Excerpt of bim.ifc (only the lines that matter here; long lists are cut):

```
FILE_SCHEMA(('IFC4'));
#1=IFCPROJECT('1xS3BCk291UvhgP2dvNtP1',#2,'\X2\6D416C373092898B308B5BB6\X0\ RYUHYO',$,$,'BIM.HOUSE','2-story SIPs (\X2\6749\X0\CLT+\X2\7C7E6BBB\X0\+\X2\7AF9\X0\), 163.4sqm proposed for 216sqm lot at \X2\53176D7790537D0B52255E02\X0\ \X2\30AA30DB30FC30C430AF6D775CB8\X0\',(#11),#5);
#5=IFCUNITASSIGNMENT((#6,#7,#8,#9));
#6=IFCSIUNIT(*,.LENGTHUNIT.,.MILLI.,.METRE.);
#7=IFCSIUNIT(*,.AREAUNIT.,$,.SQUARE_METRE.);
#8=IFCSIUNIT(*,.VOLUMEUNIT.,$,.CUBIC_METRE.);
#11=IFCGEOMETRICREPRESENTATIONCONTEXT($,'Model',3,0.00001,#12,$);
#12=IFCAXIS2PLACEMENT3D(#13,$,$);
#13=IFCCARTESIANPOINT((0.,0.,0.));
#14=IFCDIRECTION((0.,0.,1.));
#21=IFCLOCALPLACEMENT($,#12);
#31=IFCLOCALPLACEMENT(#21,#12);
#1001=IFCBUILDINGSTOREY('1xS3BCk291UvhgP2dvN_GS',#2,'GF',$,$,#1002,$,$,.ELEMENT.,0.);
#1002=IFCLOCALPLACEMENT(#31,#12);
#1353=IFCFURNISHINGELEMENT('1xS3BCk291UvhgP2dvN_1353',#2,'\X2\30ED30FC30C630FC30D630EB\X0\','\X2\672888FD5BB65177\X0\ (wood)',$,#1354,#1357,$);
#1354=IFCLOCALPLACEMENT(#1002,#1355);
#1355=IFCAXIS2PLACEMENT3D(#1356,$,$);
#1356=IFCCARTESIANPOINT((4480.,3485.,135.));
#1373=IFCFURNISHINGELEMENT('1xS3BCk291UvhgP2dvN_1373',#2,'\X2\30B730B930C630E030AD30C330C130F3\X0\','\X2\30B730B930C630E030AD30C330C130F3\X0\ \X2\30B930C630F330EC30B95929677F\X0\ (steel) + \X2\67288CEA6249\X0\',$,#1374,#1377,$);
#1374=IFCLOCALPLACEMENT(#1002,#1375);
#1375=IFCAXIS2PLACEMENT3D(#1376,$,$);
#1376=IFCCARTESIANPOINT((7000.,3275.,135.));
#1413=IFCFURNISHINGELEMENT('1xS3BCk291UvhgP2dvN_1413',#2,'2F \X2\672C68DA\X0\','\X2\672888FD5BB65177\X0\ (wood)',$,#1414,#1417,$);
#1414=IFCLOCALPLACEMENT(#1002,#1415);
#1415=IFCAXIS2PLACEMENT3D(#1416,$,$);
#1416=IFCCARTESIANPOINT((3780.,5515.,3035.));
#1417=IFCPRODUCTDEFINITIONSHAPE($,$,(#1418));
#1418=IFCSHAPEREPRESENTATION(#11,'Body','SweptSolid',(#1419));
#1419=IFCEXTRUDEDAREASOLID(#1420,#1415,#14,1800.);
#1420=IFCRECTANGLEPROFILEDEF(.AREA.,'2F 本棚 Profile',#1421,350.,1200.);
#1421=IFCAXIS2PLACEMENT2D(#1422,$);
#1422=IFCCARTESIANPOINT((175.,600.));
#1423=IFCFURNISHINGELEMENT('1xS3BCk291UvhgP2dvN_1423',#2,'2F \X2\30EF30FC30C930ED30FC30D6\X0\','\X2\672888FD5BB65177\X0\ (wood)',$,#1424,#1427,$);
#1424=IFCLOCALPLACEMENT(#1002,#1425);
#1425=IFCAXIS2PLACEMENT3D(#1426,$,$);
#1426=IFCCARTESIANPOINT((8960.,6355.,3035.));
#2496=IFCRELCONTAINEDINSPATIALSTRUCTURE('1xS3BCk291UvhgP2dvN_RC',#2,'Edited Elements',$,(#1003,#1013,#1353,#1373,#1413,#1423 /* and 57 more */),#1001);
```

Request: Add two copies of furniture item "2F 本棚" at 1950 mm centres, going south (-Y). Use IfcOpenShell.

```python
import numpy as np
import ifcopenshell
import ifcopenshell.api.geometry
import ifcopenshell.api.root
import ifcopenshell.util.element
import ifcopenshell.util.placement

model = ifcopenshell.open("bim.ifc")


def reuse_history(source, copy):
    """copy_class also copies each property set's owner history, people and application; keep the originals."""
    for rel in copy.IsDefinedBy:
        if rel.is_a("IfcRelDefinesByProperties") and (history := rel.RelatingPropertyDefinition.OwnerHistory):
            rel.RelatingPropertyDefinition.OwnerHistory = source.OwnerHistory
            ifcopenshell.util.element.remove_deep2(model, history)


source = model.by_id(1413)
base = ifcopenshell.util.placement.get_local_placement(source.ObjectPlacement)
step = np.array([0.0, -1.0, 0.0]) * 1950.0

for i in range(1, 3):
    copy = ifcopenshell.api.root.copy_class(model, product=source)
    copy.Representation = ifcopenshell.util.element.copy_deep(
        model, source.Representation, exclude=["IfcGeometricRepresentationContext", "IfcRepresentationMap"]
    )
    reuse_history(source, copy)
    matrix = base.copy()
    matrix[:3, 3] += i * step
    print("added at", matrix[:3, 3].round(3) + 0.0)
    ifcopenshell.api.geometry.edit_object_placement(model, product=copy, matrix=matrix, is_si=False)

model.write("bim_edited.ifc")
```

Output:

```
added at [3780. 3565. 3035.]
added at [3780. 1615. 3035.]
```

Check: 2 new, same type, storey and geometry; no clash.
